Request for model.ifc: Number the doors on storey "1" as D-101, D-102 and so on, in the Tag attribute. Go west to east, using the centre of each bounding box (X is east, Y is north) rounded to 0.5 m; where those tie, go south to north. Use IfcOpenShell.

First a look at what the model holds.

```python
import ifcopenshell
import ifcopenshell.util.element
import ifcopenshell.util.placement

model = ifcopenshell.open("model.ifc")
print(model.schema)
storey = next(s for s in model.by_type("IfcBuildingStorey") if s.Name == "1")
doors = [e for e in ifcopenshell.util.element.get_decomposition(storey) if e.is_a("IfcDoor")]
for e in sorted(doors, key=lambda e: e.id()):
    origin = ifcopenshell.util.placement.get_local_placement(e.ObjectPlacement)[:3, 3]
    print(e.id(), e.Tag, e.Name, origin.round(2) + 0.0, sep=" | ")
```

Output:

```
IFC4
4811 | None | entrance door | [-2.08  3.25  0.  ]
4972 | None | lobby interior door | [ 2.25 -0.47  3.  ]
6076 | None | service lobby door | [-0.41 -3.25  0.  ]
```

```python
import ifcopenshell
import ifcopenshell.geom
import ifcopenshell.util.element
import ifcopenshell.util.shape

model = ifcopenshell.open("model.ifc")
settings = ifcopenshell.geom.settings()
settings.set("use-world-coords", True)


def centre(element):
    shape = ifcopenshell.geom.create_shape(settings, element)
    return ifcopenshell.util.shape.get_bbox_centroid(shape.geometry)


storey = next(s for s in model.by_type("IfcBuildingStorey") if s.Name == "1")
doors = [e for e in ifcopenshell.util.element.get_decomposition(storey) if e.is_a("IfcDoor")]

# Insertion points can sit at a corner or the storey origin, so sort by the geometry (in metres).
centres = {e: centre(e) for e in doors}
doors.sort(key=lambda e: (round(centres[e][0] / 0.5), centres[e][1]))

for i, e in enumerate(doors, start=1):
    number = f"D-1{i:02d}"
    e.Tag = number
    print(e.id(), number)

model.write("model_rev.ifc")
```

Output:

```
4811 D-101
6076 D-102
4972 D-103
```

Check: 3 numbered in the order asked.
